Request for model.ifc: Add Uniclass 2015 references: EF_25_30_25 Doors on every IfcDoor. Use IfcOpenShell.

First a look at what the model holds.

```python
import ifcopenshell

model = ifcopenshell.open("model.ifc")
print(model.schema)
print("classifications:", [c.Name for c in model.by_type("IfcClassification")])
for ifc_class in ("IfcDoor", "IfcRoof", "IfcStair", "IfcWall", "IfcWindow"):
    print(ifc_class, len(model.by_type(ifc_class)))
```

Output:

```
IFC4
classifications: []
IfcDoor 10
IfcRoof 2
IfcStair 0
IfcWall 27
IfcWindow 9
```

```python
import ifcopenshell
import ifcopenshell.api.classification

model = ifcopenshell.open("model.ifc")

system = ifcopenshell.api.classification.add_classification(model, classification="Uniclass 2015")

codes = {
    "IfcDoor": ("EF_25_30_25", "Doors"),
}
for ifc_class, (code, name) in codes.items():
    products = model.by_type(ifc_class)
    ifcopenshell.api.classification.add_reference(
        model, products=products, classification=system, identification=code, name=name
    )
    print(code, len(products))

model.write("model_rev.ifc")
```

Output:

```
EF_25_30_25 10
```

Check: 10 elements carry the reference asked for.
